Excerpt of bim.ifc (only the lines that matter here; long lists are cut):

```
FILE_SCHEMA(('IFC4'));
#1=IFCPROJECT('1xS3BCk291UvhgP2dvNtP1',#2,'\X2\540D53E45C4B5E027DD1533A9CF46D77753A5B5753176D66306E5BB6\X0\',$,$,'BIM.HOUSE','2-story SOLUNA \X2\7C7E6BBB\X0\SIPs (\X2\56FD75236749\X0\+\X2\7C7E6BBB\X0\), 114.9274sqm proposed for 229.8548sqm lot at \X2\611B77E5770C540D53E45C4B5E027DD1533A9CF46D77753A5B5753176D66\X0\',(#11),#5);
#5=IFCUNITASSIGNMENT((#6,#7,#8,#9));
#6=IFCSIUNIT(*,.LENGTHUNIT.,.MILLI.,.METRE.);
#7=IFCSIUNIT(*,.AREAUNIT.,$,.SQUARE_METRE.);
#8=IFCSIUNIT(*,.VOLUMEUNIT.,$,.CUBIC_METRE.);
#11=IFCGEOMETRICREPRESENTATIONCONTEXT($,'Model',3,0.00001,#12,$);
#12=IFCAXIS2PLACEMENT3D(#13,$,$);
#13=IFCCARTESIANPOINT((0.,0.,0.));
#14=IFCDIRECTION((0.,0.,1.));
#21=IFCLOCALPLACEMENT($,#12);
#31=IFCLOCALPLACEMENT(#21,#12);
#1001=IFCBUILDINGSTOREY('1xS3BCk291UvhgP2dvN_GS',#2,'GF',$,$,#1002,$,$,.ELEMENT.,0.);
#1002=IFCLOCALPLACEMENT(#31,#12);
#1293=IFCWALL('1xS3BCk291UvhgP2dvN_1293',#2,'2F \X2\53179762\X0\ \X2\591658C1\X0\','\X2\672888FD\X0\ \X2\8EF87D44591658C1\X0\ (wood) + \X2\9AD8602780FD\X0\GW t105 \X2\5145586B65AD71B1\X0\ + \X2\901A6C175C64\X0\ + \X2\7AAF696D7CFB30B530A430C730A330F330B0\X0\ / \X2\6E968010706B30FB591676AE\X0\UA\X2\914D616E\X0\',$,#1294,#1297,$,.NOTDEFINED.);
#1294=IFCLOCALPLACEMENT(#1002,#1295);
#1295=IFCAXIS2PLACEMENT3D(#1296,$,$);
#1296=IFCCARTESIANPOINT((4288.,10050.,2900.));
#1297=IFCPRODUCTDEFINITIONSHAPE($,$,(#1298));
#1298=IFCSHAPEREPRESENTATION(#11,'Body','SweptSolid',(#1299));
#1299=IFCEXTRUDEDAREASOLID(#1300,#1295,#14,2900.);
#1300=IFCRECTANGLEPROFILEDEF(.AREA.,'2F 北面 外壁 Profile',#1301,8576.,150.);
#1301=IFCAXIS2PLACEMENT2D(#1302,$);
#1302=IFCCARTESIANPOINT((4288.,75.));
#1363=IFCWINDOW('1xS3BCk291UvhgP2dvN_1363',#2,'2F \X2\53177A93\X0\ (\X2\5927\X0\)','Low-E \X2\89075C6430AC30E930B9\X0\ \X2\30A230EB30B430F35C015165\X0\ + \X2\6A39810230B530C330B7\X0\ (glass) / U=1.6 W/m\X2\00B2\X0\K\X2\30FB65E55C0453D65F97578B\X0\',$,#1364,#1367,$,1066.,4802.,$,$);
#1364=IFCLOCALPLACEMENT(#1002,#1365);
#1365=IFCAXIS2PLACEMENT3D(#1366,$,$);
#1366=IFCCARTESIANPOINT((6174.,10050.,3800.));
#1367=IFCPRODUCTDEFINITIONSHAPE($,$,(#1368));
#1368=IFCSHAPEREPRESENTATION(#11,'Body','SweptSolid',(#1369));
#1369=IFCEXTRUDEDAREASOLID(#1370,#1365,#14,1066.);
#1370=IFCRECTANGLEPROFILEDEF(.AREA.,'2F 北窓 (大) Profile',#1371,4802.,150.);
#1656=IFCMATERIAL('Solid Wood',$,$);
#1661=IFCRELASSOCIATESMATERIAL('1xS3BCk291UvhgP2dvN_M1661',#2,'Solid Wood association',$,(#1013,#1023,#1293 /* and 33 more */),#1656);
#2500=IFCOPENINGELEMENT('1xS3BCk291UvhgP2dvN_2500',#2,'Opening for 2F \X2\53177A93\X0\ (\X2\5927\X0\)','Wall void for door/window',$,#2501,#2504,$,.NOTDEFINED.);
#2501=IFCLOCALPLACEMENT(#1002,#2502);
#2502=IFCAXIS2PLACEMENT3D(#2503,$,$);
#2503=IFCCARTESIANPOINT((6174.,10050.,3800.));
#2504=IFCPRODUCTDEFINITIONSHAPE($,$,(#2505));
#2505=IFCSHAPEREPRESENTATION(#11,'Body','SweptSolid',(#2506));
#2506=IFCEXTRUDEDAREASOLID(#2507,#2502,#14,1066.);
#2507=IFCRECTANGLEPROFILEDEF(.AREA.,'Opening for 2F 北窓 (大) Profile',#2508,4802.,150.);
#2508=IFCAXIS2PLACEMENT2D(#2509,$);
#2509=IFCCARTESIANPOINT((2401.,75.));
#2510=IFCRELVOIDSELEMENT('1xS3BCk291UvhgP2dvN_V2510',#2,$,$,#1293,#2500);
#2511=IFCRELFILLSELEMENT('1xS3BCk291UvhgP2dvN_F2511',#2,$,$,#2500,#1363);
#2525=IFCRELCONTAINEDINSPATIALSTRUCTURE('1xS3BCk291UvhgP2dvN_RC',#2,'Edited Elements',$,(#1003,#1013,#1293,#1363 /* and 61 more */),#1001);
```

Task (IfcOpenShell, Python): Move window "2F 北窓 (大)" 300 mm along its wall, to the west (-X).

```python
import ifcopenshell
import ifcopenshell.api.geometry
import ifcopenshell.util.placement
import ifcopenshell.util.unit

model = ifcopenshell.open("bim.ifc")
unit_scale = ifcopenshell.util.unit.calculate_unit_scale(model)

window = model.by_guid("1xS3BCk291UvhgP2dvN_1363")
opening = window.FillsVoids[0].RelatingOpeningElement
wall = opening.VoidsElements[0].RelatingBuildingElement

wall_matrix = ifcopenshell.util.placement.get_local_placement(wall.ObjectPlacement)
shift = wall_matrix[:3, 0] * -0.3 / unit_scale
before = ifcopenshell.util.placement.get_local_placement(window.ObjectPlacement)[:3, 3].copy()

# The window is not placed relative to its opening, so move both.
for product in (opening, window):
    matrix = ifcopenshell.util.placement.get_local_placement(product.ObjectPlacement)
    matrix[:3, 3] += shift
    ifcopenshell.api.geometry.edit_object_placement(model, product=product, matrix=matrix, is_si=False)

after = ifcopenshell.util.placement.get_local_placement(window.ObjectPlacement)[:3, 3]
print("window moved by", (after - before).round(3) + 0.0)

model.write("bim-out.ifc")
```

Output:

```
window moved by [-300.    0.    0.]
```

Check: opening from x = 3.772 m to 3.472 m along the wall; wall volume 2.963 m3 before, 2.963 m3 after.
